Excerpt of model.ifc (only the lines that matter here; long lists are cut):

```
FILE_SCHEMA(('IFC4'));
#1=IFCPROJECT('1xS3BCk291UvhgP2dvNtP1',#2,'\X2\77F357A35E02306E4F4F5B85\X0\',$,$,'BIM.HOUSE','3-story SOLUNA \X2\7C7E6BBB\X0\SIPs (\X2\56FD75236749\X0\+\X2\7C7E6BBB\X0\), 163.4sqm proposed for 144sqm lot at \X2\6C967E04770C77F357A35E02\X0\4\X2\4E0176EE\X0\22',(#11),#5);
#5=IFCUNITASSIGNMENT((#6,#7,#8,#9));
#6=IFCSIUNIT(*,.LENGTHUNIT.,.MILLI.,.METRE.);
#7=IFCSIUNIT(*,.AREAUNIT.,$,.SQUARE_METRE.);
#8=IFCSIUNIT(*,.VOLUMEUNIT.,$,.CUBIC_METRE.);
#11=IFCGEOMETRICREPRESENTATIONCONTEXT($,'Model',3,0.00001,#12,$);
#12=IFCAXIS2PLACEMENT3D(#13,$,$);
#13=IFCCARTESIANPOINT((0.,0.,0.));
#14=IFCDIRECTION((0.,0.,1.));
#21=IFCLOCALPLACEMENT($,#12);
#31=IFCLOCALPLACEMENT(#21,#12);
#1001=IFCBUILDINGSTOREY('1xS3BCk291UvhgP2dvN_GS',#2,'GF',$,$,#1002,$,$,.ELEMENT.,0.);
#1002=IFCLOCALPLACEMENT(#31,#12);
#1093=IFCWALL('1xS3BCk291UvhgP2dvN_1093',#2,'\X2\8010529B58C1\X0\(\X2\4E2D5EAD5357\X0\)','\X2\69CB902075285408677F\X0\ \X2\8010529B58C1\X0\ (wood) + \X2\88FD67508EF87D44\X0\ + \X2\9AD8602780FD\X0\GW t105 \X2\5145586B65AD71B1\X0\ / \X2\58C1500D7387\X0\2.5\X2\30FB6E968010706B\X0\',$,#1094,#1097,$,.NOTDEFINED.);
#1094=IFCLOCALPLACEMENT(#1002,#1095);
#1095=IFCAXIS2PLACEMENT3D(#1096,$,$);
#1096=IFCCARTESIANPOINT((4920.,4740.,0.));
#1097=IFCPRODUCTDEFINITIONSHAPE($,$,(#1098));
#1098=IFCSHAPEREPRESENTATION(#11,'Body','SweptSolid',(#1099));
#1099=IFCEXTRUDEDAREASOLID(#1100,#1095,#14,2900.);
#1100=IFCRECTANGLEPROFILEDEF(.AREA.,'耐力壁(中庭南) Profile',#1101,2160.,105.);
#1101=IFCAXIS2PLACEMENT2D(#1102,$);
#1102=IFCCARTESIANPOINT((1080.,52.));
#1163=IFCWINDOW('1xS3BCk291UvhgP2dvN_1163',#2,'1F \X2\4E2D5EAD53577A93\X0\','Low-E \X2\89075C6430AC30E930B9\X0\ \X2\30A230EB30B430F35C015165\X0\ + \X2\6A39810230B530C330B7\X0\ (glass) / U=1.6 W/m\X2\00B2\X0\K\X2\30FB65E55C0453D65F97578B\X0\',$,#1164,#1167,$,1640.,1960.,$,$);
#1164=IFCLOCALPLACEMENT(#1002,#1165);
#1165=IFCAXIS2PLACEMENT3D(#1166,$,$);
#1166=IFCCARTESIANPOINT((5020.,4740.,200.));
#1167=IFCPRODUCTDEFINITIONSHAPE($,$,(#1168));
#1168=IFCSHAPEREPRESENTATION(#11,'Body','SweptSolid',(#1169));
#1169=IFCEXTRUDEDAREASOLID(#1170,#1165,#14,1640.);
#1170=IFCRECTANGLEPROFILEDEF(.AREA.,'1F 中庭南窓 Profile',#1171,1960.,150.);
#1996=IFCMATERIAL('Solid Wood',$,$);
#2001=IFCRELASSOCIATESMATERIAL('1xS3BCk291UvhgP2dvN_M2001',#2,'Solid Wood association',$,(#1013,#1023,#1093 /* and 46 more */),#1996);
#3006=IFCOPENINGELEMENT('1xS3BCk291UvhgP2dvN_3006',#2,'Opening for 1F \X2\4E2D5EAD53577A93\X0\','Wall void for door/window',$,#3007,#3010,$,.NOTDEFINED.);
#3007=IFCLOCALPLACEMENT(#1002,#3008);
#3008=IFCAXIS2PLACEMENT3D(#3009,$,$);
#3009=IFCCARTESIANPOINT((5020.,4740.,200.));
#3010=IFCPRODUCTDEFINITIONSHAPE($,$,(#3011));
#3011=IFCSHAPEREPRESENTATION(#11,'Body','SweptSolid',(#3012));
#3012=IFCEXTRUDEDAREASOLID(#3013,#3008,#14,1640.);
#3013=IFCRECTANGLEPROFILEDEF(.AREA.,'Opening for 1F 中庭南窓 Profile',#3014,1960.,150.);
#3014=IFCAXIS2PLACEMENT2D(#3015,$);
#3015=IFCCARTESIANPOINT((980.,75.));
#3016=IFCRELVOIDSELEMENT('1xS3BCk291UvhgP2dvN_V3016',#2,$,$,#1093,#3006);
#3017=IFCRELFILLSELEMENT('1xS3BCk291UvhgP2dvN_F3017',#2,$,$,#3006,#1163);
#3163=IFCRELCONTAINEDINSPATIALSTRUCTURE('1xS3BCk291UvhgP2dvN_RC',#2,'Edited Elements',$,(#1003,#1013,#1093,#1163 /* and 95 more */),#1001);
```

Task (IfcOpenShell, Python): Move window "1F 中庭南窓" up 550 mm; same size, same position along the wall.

```python
import numpy as np
import ifcopenshell
import ifcopenshell.api.geometry
import ifcopenshell.util.placement
import ifcopenshell.util.unit

model = ifcopenshell.open("model.ifc")
unit_scale = ifcopenshell.util.unit.calculate_unit_scale(model)

window = model.by_guid("1xS3BCk291UvhgP2dvN_1163")
opening = window.FillsVoids[0].RelatingOpeningElement
dz = 0.55 / unit_scale

shift = np.array([0.0, 0.0, dz])
# The window is not placed relative to its opening, so move both.
for product in (opening, window):
    matrix = ifcopenshell.util.placement.get_local_placement(product.ObjectPlacement)
    matrix[:3, 3] += shift
    ifcopenshell.api.geometry.edit_object_placement(model, product=product, matrix=matrix, is_si=False)

print(f"moved by {dz * unit_scale:+.3f} m")

model.write("model_rev.ifc")
```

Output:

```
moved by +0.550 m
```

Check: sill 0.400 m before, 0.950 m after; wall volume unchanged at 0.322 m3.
